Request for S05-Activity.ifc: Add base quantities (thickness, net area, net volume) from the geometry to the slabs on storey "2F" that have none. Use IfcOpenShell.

First a look at what the model holds.

```python
import ifcopenshell
import ifcopenshell.util.element
import ifcopenshell.util.unit

model = ifcopenshell.open("S05-Activity.ifc")
print(model.schema)
for unit_type in ("LENGTHUNIT", "AREAUNIT", "VOLUMEUNIT"):
    print(unit_type, ifcopenshell.util.unit.calculate_unit_scale(model, unit_type))
storey = next(s for s in model.by_type("IfcBuildingStorey") if s.Name == "2F")
slabs = [e for e in ifcopenshell.util.element.get_decomposition(storey) if e.is_a("IfcSlab")]
for e in sorted(slabs, key=lambda e: e.id()):
    print(e.id(), e.is_a(), e.Name, list(ifcopenshell.util.element.get_psets(e, qtos_only=True)), sep=" | ")
```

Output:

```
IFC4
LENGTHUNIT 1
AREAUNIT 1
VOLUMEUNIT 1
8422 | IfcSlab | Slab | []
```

```python
import ifcopenshell
import ifcopenshell.api.pset
import ifcopenshell.geom
import ifcopenshell.util.element
import ifcopenshell.util.shape
import ifcopenshell.util.unit

model = ifcopenshell.open("S05-Activity.ifc")
unit_scale = ifcopenshell.util.unit.calculate_unit_scale(model)
area_scale = ifcopenshell.util.unit.calculate_unit_scale(model, "AREAUNIT")
volume_scale = ifcopenshell.util.unit.calculate_unit_scale(model, "VOLUMEUNIT")
settings = ifcopenshell.geom.settings()

storey = next(s for s in model.by_type("IfcBuildingStorey") if s.Name == "2F")
slabs = [e for e in ifcopenshell.util.element.get_decomposition(storey) if e.is_a("IfcSlab")]

for e in sorted(slabs, key=lambda e: e.id()):
    if ifcopenshell.util.element.get_psets(e, qtos_only=True, should_inherit=False):
        continue
    # Geometry comes back in metres, in the element's own axes.
    shape = ifcopenshell.geom.create_shape(settings, e)
    values = {
        "Width": ifcopenshell.util.shape.get_z(shape.geometry) / unit_scale,
        "NetArea": ifcopenshell.util.shape.get_footprint_area(shape.geometry) / area_scale,
        "NetVolume": ifcopenshell.util.shape.get_volume(shape.geometry) / volume_scale,
    }
    qto = ifcopenshell.api.pset.add_qto(model, product=e, name="Qto_SlabBaseQuantities")
    ifcopenshell.api.pset.edit_qto(model, qto=qto, properties=values)
    print(e.id(), {k: round(v, 3) for k, v in values.items()})

model.write("S05-Activity_edited.ifc")
```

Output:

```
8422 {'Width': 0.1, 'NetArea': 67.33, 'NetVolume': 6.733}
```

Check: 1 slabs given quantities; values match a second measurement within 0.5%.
